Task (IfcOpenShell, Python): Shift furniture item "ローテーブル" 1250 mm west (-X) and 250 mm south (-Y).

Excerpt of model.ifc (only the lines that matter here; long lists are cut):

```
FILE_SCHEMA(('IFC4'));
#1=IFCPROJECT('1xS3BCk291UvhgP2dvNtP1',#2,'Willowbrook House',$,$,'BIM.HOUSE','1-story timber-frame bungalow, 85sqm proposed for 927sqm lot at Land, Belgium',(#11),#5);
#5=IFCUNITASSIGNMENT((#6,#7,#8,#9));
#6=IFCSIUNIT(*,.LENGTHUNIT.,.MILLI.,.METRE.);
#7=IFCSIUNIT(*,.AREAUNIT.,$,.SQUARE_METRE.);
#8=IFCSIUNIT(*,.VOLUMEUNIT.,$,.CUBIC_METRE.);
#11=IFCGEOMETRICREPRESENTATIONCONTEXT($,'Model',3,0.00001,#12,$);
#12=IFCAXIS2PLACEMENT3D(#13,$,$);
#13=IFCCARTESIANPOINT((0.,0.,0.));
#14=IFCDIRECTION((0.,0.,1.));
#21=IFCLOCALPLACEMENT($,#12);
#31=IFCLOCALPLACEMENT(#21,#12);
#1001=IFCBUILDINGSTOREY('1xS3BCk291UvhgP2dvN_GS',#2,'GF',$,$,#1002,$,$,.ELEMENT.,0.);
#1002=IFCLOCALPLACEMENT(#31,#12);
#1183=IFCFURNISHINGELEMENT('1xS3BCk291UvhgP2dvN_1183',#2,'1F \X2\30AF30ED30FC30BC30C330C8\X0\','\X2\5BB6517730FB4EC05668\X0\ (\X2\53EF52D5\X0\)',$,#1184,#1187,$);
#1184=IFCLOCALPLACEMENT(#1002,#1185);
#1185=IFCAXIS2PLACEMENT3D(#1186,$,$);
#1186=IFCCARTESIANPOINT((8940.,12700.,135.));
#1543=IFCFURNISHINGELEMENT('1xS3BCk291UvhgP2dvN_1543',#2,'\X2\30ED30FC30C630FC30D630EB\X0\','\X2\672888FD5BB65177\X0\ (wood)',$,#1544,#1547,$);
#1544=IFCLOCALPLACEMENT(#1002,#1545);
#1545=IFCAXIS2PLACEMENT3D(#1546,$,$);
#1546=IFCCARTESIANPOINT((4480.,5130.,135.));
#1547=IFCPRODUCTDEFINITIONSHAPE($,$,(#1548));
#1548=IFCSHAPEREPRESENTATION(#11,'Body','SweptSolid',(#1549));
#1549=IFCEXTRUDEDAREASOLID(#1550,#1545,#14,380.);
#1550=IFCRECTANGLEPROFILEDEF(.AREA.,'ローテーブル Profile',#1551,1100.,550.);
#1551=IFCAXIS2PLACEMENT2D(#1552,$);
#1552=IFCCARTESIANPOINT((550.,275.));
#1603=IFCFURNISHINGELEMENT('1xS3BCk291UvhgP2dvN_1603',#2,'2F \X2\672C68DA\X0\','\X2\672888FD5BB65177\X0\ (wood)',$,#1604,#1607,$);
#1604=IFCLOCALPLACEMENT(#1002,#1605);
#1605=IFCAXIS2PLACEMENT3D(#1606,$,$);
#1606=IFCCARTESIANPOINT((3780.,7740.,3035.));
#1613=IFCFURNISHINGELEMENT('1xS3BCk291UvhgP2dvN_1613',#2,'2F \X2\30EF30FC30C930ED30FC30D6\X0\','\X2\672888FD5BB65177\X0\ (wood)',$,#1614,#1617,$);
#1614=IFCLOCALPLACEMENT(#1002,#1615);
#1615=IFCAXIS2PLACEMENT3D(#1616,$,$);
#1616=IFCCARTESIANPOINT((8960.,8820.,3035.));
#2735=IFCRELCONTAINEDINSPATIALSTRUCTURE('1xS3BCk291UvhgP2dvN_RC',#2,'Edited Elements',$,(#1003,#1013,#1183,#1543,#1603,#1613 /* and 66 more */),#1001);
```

```python
import ifcopenshell
import ifcopenshell.api.geometry
import ifcopenshell.util.placement
import ifcopenshell.util.unit

model = ifcopenshell.open("model.ifc")
unit_scale = ifcopenshell.util.unit.calculate_unit_scale(model)

item = model.by_id(1543)
matrix = ifcopenshell.util.placement.get_local_placement(item.ObjectPlacement)
matrix[0, 3] -= 1.25 / unit_scale
matrix[1, 3] -= 0.25 / unit_scale
ifcopenshell.api.geometry.edit_object_placement(model, product=item, matrix=matrix, is_si=False)

print(ifcopenshell.util.placement.get_local_placement(item.ObjectPlacement).round(3) + 0.0)

model.write("model_rev.ifc")
```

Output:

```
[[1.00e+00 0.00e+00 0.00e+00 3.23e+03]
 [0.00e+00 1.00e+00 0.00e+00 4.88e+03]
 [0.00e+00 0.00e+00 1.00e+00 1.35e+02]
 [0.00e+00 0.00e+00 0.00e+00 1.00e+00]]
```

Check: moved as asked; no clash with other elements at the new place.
